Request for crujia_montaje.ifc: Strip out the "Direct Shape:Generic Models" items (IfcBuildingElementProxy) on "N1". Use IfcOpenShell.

First a look at what the model holds.

```python
import ifcopenshell
import ifcopenshell.util.element

model = ifcopenshell.open("crujia_montaje.ifc")
print(model.schema)
storey = next(s for s in model.by_type("IfcBuildingStorey") if s.Name == "N1")
proxies = [e for e in ifcopenshell.util.element.get_decomposition(storey) if e.is_a("IfcBuildingElementProxy")]
seen = {}
for e in proxies:
    element_type = ifcopenshell.util.element.get_type(e)
    name = element_type.Name if element_type not in (None, e) else None
    seen[name] = seen.get(name, 0) + 1
for name, count in sorted(seen.items(), key=str):
    print(count, "x", name)
```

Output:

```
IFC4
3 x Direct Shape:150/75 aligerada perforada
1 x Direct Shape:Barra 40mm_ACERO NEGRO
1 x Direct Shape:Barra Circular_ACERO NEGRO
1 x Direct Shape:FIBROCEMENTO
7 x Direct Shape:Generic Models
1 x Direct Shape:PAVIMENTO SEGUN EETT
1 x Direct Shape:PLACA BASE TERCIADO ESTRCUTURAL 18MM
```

```python
import ifcopenshell
import ifcopenshell.api.root
import ifcopenshell.util.element

model = ifcopenshell.open("crujia_montaje.ifc")

storey = next(s for s in model.by_type("IfcBuildingStorey") if s.Name == "N1")
proxies = [e for e in ifcopenshell.util.element.get_decomposition(storey) if e.is_a("IfcBuildingElementProxy")]
targets = [e for e in proxies if (t := ifcopenshell.util.element.get_type(e)) not in (None, e) and t.Name == "Direct Shape:Generic Models"]

for e in targets:
    ifcopenshell.api.root.remove_product(model, product=e)
print(len(targets), "removed")

model.write("crujia_montaje_rev.ifc")
```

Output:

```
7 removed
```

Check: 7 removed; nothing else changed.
